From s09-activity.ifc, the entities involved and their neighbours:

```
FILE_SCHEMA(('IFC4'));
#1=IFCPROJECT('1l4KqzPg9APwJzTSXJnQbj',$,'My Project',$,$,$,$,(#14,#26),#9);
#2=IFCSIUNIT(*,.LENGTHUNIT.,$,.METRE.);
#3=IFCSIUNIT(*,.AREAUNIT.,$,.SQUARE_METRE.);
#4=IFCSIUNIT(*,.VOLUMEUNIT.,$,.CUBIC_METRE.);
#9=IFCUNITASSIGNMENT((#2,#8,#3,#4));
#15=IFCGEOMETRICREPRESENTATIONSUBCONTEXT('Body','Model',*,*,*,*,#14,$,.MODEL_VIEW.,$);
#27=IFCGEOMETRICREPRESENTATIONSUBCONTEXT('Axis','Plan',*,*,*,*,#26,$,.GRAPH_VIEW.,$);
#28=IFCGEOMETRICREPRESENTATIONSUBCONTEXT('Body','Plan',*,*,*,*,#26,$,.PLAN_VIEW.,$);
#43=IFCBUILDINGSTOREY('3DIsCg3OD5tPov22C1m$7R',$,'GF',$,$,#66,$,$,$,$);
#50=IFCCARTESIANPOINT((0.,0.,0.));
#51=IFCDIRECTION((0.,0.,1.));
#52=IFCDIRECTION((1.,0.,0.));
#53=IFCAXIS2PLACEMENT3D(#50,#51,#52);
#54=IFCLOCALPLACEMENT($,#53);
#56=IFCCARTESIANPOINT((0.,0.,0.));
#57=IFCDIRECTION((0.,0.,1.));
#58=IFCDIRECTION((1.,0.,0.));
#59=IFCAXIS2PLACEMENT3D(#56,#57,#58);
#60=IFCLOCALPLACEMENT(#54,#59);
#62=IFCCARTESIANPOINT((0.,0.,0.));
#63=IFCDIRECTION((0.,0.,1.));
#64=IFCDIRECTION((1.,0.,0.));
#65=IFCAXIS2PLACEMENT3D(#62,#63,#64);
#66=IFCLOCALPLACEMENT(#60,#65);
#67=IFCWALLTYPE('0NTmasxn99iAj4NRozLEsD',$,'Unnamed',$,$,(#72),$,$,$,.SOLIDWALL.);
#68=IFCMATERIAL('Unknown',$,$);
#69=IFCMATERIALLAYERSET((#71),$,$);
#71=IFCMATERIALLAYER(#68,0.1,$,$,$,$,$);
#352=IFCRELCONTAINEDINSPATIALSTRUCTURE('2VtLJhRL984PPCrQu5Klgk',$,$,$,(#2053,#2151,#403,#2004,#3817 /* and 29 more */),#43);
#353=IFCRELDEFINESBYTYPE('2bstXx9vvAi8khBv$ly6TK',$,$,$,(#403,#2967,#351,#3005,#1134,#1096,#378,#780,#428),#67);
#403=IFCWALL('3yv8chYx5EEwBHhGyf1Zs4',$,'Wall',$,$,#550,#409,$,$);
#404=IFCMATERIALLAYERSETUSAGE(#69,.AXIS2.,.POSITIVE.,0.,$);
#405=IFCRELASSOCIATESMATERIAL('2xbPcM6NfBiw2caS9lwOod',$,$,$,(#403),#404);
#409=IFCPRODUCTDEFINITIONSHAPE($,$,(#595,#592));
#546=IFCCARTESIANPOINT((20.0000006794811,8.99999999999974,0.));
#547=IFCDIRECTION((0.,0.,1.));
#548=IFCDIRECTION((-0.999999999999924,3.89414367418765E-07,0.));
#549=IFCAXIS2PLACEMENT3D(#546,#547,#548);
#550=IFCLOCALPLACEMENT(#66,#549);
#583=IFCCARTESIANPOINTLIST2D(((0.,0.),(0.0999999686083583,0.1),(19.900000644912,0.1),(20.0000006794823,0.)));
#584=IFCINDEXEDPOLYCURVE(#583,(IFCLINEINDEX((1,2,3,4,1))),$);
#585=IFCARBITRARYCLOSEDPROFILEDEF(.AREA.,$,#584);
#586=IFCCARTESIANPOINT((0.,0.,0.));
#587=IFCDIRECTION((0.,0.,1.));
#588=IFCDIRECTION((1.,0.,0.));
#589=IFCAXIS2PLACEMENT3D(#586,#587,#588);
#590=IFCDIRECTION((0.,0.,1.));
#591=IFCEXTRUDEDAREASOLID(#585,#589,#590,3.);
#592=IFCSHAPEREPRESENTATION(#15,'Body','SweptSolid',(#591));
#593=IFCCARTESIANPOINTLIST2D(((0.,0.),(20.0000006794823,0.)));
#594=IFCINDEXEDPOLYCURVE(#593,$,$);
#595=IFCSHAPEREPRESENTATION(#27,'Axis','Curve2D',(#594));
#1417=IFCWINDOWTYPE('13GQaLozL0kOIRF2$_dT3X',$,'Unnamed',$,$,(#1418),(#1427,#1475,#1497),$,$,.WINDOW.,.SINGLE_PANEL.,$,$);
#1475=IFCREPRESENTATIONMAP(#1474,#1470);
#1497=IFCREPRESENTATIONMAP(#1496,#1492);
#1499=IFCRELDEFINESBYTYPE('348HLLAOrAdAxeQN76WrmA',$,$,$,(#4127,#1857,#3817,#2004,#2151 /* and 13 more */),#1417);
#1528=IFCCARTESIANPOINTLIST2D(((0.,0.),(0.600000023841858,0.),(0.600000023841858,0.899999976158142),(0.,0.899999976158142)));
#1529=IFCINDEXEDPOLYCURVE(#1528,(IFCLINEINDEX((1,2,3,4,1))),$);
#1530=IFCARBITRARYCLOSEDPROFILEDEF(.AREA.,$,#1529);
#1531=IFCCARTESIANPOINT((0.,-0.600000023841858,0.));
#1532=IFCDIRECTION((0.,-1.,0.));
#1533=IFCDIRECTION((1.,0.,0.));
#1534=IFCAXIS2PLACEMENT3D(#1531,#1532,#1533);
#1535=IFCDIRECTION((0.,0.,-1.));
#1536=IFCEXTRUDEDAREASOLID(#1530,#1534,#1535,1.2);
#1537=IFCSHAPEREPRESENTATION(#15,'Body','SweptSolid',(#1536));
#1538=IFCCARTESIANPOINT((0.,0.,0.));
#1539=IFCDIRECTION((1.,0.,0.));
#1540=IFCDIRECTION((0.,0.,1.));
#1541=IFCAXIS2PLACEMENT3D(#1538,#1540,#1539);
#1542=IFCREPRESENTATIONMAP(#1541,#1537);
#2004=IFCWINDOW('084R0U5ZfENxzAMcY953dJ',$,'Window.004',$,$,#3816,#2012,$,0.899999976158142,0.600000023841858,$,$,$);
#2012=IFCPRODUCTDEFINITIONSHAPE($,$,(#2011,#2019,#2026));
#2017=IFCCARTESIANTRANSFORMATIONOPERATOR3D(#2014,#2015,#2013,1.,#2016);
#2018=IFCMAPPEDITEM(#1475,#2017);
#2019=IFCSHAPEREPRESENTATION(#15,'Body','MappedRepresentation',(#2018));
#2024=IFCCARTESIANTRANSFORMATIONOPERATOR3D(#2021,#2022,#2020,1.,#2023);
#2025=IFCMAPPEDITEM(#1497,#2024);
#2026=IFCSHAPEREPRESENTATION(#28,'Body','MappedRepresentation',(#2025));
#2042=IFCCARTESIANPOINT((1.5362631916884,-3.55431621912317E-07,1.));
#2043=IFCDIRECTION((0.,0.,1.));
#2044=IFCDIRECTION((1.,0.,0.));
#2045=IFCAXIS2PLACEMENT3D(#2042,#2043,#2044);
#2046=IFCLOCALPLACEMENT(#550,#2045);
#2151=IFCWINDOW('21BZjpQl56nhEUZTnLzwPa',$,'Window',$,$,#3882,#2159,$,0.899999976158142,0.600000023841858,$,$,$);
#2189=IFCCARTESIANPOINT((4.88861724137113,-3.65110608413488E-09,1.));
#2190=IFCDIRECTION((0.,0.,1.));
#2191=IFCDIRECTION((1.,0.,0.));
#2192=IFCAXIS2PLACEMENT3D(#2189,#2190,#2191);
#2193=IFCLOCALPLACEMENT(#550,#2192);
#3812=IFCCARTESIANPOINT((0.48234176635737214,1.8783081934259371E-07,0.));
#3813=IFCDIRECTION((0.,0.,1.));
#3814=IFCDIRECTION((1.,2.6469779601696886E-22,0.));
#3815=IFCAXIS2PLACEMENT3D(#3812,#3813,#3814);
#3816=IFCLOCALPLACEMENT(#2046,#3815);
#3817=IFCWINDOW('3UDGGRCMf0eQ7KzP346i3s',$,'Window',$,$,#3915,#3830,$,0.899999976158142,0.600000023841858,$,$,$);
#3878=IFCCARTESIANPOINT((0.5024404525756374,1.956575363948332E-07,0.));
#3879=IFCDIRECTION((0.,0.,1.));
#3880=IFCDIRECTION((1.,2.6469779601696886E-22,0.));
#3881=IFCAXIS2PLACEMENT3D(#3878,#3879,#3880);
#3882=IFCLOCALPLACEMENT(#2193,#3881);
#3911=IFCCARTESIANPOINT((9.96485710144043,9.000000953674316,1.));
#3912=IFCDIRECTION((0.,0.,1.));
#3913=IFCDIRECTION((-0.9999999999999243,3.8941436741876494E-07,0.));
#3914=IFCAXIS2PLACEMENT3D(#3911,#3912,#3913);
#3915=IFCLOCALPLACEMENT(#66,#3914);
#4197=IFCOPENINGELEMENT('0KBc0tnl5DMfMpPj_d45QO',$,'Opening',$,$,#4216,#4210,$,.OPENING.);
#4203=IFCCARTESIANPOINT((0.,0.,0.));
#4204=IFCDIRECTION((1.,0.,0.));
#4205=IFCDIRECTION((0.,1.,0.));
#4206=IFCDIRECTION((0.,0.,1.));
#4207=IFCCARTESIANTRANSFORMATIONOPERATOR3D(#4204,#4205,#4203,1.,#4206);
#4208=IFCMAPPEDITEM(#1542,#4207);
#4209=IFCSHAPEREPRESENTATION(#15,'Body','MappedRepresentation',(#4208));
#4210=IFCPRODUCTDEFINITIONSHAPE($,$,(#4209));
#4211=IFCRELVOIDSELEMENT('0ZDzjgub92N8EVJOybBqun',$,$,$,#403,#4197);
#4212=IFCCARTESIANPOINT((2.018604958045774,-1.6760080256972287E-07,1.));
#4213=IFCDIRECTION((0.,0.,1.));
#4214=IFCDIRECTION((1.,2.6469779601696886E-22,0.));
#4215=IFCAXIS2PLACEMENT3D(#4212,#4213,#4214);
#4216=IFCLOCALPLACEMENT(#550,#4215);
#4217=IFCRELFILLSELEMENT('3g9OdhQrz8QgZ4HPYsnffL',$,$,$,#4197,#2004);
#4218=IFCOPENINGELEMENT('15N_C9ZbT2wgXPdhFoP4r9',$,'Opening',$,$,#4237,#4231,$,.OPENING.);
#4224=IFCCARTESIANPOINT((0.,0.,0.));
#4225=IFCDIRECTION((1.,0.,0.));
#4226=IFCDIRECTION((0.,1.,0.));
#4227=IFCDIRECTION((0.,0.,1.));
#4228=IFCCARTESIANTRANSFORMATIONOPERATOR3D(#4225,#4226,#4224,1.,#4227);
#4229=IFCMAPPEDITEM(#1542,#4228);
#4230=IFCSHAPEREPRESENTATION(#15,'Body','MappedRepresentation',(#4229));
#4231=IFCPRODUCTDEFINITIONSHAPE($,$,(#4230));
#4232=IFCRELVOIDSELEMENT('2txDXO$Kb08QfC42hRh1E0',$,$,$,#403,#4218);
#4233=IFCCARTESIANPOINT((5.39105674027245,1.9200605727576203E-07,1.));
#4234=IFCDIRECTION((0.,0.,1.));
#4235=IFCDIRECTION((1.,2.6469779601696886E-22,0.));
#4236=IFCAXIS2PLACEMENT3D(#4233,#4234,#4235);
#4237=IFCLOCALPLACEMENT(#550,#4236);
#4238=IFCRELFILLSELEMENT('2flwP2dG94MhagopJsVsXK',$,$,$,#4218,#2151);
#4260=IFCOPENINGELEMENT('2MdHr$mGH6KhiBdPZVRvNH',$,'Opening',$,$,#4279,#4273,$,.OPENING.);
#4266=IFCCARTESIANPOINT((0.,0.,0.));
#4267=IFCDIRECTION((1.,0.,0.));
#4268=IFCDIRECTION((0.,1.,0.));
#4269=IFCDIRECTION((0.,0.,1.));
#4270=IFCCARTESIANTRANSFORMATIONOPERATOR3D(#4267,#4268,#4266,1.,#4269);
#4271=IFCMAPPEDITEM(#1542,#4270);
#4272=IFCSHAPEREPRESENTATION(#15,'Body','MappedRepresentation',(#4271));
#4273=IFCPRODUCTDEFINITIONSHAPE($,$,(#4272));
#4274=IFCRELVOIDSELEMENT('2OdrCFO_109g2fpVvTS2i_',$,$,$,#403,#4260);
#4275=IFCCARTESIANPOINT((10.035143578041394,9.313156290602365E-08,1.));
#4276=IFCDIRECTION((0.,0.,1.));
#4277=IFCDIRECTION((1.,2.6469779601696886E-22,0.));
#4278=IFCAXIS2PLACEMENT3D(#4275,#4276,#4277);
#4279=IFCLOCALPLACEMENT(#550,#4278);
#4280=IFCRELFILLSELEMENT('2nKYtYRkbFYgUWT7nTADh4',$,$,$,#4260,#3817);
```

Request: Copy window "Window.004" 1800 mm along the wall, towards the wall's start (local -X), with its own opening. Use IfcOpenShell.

```python
import ifcopenshell
import ifcopenshell.api.feature
import ifcopenshell.api.geometry
import ifcopenshell.api.root
import ifcopenshell.geom
import ifcopenshell.util.element
import ifcopenshell.util.placement
import ifcopenshell.util.shape

model = ifcopenshell.open("s09-activity.ifc")
settings = ifcopenshell.geom.settings()


def volume(element):
    """Net volume in cubic metres, openings subtracted."""
    shape = ifcopenshell.geom.create_shape(settings, element)
    return ifcopenshell.util.shape.get_volume(shape.geometry)


window = model.by_guid("084R0U5ZfENxzAMcY953dJ")
opening = window.FillsVoids[0].RelatingOpeningElement
wall = opening.VoidsElements[0].RelatingBuildingElement
before = volume(wall)
shift = ifcopenshell.util.placement.get_local_placement(wall.ObjectPlacement)[:3, 0] * -1.8

# copy_class copies the void relationship, type, container and properties, but no geometry.
new_opening = ifcopenshell.api.root.copy_class(model, product=opening)
new_opening.Representation = ifcopenshell.util.element.copy_deep(
    model, opening.Representation, exclude=["IfcGeometricRepresentationContext", "IfcRepresentationMap"]
)
new_window = ifcopenshell.api.root.copy_class(model, product=window)
new_window.Representation = ifcopenshell.util.element.copy_deep(
    model, window.Representation, exclude=["IfcGeometricRepresentationContext", "IfcRepresentationMap"]
)
ifcopenshell.api.feature.add_filling(model, opening=new_opening, element=new_window)

for old, new in ((opening, new_opening), (window, new_window)):
    matrix = ifcopenshell.util.placement.get_local_placement(old.ObjectPlacement)
    matrix[:3, 3] += shift
    ifcopenshell.api.geometry.edit_object_placement(model, product=new, matrix=matrix, is_si=False)

after = volume(wall)

print(f"wall volume {before:.3f} -> {after:.3f} m3")

model.write("s09-activity-out.ifc")
```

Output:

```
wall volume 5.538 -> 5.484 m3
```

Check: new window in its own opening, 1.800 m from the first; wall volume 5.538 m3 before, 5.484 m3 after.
